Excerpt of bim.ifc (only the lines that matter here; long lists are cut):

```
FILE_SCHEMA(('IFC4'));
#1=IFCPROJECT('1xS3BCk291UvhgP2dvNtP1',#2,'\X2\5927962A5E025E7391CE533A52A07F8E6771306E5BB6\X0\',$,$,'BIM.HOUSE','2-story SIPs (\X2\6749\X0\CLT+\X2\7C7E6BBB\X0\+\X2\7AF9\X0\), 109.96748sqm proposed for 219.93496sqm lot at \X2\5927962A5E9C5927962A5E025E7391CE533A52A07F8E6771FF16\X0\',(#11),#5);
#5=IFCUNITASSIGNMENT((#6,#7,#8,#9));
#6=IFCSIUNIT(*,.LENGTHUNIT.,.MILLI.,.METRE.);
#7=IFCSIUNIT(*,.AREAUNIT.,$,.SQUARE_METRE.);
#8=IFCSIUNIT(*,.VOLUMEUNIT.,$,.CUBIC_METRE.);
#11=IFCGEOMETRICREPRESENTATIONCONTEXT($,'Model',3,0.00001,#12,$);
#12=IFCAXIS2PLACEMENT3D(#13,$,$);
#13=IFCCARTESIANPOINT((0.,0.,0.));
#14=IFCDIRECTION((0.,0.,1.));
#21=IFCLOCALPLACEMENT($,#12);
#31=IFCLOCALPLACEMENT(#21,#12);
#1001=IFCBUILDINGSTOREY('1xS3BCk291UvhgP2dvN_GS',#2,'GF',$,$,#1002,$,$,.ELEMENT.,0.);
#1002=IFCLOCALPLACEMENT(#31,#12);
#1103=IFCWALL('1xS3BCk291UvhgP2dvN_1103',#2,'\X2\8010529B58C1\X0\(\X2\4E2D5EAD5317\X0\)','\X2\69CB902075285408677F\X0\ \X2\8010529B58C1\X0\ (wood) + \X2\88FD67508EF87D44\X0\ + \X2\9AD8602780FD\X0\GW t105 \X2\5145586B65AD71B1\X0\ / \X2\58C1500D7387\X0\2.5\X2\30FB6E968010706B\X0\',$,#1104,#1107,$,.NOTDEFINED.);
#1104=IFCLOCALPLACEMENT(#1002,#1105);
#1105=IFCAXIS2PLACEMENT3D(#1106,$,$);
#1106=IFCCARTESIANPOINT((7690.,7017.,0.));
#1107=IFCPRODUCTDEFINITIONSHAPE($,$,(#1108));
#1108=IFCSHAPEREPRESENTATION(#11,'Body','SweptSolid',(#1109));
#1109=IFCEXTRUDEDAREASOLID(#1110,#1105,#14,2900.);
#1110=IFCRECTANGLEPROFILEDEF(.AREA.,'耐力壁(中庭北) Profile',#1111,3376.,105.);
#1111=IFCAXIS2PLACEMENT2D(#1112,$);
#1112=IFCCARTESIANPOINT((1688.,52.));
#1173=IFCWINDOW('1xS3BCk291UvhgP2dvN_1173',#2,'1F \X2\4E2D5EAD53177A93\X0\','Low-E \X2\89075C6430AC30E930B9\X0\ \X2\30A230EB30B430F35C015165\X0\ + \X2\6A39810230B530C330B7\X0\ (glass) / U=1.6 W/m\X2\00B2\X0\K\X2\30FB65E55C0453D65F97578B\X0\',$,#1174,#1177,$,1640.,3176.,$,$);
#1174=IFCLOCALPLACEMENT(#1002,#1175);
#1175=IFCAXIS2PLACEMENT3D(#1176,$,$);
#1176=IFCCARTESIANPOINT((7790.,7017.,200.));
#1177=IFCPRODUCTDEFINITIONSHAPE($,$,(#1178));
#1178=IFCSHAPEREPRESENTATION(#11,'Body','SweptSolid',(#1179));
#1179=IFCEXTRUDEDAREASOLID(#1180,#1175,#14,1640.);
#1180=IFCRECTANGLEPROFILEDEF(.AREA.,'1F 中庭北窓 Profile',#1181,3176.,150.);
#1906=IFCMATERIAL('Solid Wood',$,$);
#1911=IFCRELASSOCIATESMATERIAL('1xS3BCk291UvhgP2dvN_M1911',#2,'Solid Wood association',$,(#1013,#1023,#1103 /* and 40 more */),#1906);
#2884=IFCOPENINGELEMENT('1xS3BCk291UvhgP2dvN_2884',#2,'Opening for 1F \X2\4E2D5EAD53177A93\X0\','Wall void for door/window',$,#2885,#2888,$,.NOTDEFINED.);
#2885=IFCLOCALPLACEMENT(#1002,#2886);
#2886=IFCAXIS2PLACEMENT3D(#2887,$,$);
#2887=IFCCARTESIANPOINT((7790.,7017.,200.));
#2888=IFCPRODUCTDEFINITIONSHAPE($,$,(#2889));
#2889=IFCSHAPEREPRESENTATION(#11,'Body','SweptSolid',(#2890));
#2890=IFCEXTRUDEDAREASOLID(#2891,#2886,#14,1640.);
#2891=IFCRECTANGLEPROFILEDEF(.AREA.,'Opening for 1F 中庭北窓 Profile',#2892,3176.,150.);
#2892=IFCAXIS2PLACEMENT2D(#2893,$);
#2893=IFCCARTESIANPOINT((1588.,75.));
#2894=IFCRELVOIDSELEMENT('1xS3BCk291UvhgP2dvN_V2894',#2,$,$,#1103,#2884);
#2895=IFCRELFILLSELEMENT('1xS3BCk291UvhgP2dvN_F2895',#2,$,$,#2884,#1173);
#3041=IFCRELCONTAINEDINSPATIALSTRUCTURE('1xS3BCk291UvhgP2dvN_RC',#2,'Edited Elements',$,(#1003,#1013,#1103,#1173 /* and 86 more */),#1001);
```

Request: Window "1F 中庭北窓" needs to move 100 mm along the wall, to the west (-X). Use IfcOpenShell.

```python
import ifcopenshell
import ifcopenshell.api.geometry
import ifcopenshell.util.placement
import ifcopenshell.util.unit

model = ifcopenshell.open("bim.ifc")
unit_scale = ifcopenshell.util.unit.calculate_unit_scale(model)

window = model.by_guid("1xS3BCk291UvhgP2dvN_1173")
opening = window.FillsVoids[0].RelatingOpeningElement
wall = opening.VoidsElements[0].RelatingBuildingElement

wall_matrix = ifcopenshell.util.placement.get_local_placement(wall.ObjectPlacement)
shift = wall_matrix[:3, 0] * -0.1 / unit_scale
before = ifcopenshell.util.placement.get_local_placement(window.ObjectPlacement)[:3, 3].copy()

# The window is not placed relative to its opening, so move both.
for product in (opening, window):
    matrix = ifcopenshell.util.placement.get_local_placement(product.ObjectPlacement)
    matrix[:3, 3] += shift
    ifcopenshell.api.geometry.edit_object_placement(model, product=product, matrix=matrix, is_si=False)

after = ifcopenshell.util.placement.get_local_placement(window.ObjectPlacement)[:3, 3]
print("window moved by", (after - before).round(3) + 0.0)

model.write("bim_v2.ifc")
```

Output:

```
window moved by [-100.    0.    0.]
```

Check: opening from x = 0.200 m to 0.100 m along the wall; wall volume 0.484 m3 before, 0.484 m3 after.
